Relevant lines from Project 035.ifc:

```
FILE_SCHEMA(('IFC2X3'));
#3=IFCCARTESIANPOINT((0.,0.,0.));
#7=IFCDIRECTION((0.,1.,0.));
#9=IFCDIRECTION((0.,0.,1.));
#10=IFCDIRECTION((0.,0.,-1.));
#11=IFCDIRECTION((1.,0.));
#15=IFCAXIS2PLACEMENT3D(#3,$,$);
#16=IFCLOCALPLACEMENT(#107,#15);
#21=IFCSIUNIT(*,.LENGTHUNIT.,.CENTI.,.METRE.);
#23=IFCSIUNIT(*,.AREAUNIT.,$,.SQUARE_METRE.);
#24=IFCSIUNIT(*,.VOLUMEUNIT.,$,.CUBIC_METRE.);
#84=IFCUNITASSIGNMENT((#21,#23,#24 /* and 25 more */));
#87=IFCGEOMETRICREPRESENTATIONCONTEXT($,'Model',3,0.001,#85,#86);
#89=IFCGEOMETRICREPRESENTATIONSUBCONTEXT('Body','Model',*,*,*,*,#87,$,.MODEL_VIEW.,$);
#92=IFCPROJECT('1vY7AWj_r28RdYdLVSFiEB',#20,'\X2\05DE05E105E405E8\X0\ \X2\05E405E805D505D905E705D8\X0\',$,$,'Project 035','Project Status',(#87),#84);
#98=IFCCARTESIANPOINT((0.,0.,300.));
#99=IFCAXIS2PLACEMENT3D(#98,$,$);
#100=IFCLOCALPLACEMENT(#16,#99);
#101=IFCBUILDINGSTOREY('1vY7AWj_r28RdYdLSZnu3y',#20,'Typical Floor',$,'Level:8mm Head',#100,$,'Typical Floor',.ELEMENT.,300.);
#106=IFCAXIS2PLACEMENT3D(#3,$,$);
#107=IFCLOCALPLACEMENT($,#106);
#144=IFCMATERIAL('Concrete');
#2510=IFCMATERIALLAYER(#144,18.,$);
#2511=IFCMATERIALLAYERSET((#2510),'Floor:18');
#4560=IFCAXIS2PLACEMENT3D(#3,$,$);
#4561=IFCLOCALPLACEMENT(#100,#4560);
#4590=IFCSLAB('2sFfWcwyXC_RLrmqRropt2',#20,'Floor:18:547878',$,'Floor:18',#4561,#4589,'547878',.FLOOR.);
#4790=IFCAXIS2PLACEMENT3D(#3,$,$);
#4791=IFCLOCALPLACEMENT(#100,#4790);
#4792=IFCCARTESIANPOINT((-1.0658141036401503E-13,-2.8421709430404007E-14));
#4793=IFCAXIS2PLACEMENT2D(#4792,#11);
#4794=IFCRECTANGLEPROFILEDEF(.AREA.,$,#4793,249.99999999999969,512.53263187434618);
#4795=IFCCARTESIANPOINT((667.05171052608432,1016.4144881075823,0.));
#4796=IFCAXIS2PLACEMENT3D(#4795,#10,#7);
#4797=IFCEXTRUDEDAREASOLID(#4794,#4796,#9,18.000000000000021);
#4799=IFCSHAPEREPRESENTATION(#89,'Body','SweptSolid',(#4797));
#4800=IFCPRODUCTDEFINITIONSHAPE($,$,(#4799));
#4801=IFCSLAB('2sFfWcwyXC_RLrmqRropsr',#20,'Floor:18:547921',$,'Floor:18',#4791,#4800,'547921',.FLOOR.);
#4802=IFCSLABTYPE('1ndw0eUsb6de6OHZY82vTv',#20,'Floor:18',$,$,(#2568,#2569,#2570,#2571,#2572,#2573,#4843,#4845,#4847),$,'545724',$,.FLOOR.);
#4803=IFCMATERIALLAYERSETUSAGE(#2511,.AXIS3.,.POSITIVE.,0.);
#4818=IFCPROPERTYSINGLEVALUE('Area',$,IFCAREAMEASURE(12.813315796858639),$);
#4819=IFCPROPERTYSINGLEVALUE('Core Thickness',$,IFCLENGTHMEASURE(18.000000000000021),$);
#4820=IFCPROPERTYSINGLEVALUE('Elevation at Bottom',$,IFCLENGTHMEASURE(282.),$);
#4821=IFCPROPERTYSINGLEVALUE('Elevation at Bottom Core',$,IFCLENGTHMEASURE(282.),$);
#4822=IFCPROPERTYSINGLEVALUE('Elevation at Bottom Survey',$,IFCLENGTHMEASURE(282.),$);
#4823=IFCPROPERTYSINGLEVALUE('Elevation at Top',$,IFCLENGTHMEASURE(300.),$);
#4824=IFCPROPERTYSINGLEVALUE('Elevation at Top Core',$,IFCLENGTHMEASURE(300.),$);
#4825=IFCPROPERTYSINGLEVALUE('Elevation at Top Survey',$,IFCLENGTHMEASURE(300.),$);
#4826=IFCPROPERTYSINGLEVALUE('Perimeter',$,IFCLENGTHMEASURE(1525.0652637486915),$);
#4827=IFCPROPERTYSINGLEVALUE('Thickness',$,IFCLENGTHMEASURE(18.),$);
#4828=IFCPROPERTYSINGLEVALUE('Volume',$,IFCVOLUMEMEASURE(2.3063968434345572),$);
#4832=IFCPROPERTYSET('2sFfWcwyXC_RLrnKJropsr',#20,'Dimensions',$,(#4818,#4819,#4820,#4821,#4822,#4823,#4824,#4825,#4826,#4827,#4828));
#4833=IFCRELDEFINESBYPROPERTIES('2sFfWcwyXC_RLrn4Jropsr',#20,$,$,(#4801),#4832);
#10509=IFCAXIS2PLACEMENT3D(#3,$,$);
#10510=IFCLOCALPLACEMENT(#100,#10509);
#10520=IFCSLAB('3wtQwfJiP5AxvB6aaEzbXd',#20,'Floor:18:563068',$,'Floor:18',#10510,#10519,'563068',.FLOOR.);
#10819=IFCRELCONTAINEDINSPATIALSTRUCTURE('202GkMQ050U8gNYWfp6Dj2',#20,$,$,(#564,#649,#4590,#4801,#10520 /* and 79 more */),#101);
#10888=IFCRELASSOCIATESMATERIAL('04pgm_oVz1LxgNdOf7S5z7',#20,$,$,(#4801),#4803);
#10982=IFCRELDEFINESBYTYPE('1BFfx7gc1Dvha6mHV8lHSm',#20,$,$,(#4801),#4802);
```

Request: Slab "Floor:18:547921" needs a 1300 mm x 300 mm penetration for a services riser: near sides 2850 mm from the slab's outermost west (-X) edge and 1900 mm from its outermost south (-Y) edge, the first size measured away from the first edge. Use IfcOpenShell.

```python
import numpy as np
import ifcopenshell
import ifcopenshell.api.feature
import ifcopenshell.api.geometry
import ifcopenshell.api.pset
import ifcopenshell.api.root
import ifcopenshell.geom
import ifcopenshell.util.element
import ifcopenshell.util.placement
import ifcopenshell.util.representation
import ifcopenshell.util.shape
import ifcopenshell.util.unit

model = ifcopenshell.open("Project 035.ifc")
unit_scale = ifcopenshell.util.unit.calculate_unit_scale(model)
area_scale = ifcopenshell.util.unit.calculate_unit_scale(model, "AREAUNIT")
volume_scale = ifcopenshell.util.unit.calculate_unit_scale(model, "VOLUMEUNIT")
settings = ifcopenshell.geom.settings()


def volume(element):
    """Net volume in cubic metres, openings subtracted."""
    shape = ifcopenshell.geom.create_shape(settings, element)
    return ifcopenshell.util.shape.get_volume(shape.geometry)


slab = model.by_guid("2sFfWcwyXC_RLrmqRropsr")
before = volume(slab)

# Extent in the slab's own axes, in metres. The edges named are its -X and -Y sides.
slab_shape = ifcopenshell.geom.create_shape(settings, slab)
vertices = ifcopenshell.util.shape.get_vertices(slab_shape.geometry)
x_min, y_min, bottom = vertices.min(axis=0)
top = vertices[:, 2].max()

opening = ifcopenshell.api.root.create_entity(model, ifc_class="IfcOpeningElement", name="Services riser opening")
context = ifcopenshell.util.representation.get_context(model, "Model", "Body", "MODEL_VIEW")
width, depth = 1.3, 0.3
outline = [(0.0, 0.0), (width, 0.0), (width, depth), (0.0, depth), (0.0, 0.0)]
# Overshoot both faces by 50 mm so the cut is clean.
shape = ifcopenshell.api.geometry.add_slab_representation(
    model, context=context, depth=top - bottom + 0.1, polyline=outline
)
ifcopenshell.api.geometry.assign_representation(model, product=opening, representation=shape)

matrix = ifcopenshell.util.placement.get_local_placement(slab.ObjectPlacement)
matrix[:, 3] = matrix @ np.append(np.array([x_min + 2.85, y_min + 1.9, bottom - 0.05]) / unit_scale, 1.0)
ifcopenshell.api.geometry.edit_object_placement(model, product=opening, matrix=matrix, is_si=False)
ifcopenshell.api.feature.add_feature(model, feature=opening, element=slab)

after = volume(slab)

# Update the slab's stored quantities.
pset = model.by_id(ifcopenshell.util.element.get_pset(slab, "Dimensions", should_inherit=False)["id"])
ifcopenshell.api.pset.edit_pset(model, pset=pset, properties={
    "Area": model.create_entity("IfcAreaMeasure", after / (top - bottom) / area_scale),
    "Volume": model.create_entity("IfcVolumeMeasure", after / volume_scale),
})

print(f"slab volume {before:.3f} -> {after:.3f} m3")

model.write("Project 035_v2.ifc")
```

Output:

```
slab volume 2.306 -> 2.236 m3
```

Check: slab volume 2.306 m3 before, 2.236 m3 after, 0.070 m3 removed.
